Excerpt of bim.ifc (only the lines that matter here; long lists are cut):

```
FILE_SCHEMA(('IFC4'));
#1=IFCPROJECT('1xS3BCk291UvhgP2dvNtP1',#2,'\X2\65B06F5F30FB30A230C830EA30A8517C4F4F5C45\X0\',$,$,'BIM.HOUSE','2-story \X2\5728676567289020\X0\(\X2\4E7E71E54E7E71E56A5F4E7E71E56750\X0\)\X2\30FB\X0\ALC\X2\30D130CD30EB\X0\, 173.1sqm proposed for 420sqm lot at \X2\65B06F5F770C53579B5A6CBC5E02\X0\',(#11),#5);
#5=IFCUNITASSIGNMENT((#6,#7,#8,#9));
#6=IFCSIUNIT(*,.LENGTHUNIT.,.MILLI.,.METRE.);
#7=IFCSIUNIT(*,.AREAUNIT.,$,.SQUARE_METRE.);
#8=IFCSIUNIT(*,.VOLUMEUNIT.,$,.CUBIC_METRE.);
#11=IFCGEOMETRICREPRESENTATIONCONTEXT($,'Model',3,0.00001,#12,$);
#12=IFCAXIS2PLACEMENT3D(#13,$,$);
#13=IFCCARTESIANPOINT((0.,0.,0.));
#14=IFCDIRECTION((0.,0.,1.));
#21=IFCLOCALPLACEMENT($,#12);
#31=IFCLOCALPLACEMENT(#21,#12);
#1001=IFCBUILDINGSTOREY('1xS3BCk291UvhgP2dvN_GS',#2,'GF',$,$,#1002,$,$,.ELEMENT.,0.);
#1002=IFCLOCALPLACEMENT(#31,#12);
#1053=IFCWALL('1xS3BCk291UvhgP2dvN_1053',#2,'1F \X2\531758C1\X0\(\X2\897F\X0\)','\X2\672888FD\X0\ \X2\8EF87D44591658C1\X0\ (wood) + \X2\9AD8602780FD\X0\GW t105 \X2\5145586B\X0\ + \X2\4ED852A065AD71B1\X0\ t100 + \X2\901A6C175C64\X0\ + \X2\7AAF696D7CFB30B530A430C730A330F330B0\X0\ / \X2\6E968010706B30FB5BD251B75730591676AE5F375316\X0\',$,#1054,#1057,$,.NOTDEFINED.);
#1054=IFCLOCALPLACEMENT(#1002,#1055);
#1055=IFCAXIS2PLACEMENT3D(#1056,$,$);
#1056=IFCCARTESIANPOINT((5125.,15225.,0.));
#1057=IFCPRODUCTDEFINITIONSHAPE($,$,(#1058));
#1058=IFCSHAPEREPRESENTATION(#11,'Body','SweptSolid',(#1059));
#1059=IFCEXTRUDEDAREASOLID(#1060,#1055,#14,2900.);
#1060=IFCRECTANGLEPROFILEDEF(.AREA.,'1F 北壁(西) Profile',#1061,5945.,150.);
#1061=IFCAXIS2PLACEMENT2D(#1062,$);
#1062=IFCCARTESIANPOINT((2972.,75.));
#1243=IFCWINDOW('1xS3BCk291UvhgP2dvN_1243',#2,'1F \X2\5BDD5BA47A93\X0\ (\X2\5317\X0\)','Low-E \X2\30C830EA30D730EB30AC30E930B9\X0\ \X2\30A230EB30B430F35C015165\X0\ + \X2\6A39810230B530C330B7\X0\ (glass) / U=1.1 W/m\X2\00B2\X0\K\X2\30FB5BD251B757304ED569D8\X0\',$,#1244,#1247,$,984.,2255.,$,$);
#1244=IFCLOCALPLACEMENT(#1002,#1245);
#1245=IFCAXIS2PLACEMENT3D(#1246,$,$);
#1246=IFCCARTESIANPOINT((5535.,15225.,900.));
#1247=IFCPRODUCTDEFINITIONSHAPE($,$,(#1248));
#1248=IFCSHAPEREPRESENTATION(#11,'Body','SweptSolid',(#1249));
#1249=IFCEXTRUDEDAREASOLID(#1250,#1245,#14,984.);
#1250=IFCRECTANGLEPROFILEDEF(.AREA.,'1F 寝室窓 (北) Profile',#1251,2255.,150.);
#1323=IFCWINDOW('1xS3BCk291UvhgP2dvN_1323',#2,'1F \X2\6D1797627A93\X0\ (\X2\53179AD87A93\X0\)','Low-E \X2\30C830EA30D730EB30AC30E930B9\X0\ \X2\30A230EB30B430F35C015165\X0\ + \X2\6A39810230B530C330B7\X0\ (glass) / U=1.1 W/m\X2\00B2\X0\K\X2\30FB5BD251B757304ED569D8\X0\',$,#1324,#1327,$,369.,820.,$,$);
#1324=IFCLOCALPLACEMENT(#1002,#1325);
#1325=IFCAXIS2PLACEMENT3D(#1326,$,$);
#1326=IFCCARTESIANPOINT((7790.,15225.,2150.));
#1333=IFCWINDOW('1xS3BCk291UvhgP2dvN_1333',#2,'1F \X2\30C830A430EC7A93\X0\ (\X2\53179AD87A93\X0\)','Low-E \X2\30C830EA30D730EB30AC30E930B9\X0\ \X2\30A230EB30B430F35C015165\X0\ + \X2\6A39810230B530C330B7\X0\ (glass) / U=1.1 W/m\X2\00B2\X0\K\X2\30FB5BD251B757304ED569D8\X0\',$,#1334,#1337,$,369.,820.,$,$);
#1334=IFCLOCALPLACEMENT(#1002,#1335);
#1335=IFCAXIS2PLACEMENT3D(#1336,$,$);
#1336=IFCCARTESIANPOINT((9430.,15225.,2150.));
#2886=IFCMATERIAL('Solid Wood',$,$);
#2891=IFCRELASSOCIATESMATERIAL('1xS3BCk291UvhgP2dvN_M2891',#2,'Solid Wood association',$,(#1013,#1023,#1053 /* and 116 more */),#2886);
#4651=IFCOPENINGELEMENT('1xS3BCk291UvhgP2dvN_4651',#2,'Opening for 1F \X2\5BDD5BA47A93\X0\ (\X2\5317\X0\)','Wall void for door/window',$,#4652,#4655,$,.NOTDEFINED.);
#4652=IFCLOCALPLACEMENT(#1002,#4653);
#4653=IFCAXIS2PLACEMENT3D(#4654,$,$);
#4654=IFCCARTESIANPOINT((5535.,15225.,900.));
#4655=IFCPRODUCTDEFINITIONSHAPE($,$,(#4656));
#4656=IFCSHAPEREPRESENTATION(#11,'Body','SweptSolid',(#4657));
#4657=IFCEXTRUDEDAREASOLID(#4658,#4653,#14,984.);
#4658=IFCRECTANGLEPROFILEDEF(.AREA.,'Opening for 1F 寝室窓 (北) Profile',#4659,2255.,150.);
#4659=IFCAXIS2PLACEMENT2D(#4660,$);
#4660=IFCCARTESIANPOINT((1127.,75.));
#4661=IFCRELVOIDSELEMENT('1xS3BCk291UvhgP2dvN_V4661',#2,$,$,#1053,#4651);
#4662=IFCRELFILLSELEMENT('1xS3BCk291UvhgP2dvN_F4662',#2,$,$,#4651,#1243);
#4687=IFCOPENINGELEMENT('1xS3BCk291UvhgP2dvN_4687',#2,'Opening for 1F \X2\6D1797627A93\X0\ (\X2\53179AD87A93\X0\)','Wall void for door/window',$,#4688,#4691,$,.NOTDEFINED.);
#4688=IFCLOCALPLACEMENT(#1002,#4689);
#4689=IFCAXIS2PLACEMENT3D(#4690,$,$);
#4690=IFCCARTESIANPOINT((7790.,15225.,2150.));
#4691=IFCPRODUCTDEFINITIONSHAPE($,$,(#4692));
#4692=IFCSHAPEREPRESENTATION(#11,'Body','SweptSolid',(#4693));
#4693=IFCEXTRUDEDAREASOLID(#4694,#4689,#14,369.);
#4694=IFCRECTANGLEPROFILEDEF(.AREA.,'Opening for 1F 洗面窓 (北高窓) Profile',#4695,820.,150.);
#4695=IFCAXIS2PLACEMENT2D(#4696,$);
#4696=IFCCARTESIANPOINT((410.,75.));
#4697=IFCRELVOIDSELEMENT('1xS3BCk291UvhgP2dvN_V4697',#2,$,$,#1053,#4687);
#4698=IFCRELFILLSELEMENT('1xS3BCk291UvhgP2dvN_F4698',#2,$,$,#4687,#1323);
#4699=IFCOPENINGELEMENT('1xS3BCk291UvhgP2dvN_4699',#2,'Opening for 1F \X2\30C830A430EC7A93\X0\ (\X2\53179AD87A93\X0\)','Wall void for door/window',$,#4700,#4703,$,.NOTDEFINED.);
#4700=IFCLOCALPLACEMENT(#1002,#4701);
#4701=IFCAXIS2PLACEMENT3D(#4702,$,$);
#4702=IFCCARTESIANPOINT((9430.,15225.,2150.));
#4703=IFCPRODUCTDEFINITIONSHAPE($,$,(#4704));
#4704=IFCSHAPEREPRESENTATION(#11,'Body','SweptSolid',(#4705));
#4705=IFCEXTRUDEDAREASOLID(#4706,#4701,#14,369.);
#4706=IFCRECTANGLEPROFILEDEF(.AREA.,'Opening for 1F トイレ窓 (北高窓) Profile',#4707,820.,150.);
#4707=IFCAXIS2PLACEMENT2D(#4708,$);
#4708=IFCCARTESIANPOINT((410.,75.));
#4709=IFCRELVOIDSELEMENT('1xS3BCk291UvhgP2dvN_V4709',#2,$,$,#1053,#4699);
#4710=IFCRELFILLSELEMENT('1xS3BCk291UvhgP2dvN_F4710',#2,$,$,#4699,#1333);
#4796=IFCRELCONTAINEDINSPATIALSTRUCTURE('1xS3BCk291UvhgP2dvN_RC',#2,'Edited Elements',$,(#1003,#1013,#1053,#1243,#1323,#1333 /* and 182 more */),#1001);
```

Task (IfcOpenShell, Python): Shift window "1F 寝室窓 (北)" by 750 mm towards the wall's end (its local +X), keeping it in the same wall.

```python
import ifcopenshell
import ifcopenshell.api.geometry
import ifcopenshell.util.placement

model = ifcopenshell.open("bim.ifc")

window = model.by_id(1243)
opening = window.FillsVoids[0].RelatingOpeningElement
wall = opening.VoidsElements[0].RelatingBuildingElement

wall_matrix = ifcopenshell.util.placement.get_local_placement(wall.ObjectPlacement)
shift = wall_matrix[:3, 0] * 750.0
before = ifcopenshell.util.placement.get_local_placement(window.ObjectPlacement)[:3, 3].copy()

# The window is not placed relative to its opening, so move both.
for product in (opening, window):
    matrix = ifcopenshell.util.placement.get_local_placement(product.ObjectPlacement)
    matrix[:3, 3] += shift
    ifcopenshell.api.geometry.edit_object_placement(model, product=product, matrix=matrix, is_si=False)

after = ifcopenshell.util.placement.get_local_placement(window.ObjectPlacement)[:3, 3]
print("window moved by", (after - before).round(3) + 0.0)

model.write("bim_rev.ifc")
```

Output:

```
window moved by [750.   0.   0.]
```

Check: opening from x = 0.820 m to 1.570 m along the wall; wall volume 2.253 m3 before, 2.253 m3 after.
